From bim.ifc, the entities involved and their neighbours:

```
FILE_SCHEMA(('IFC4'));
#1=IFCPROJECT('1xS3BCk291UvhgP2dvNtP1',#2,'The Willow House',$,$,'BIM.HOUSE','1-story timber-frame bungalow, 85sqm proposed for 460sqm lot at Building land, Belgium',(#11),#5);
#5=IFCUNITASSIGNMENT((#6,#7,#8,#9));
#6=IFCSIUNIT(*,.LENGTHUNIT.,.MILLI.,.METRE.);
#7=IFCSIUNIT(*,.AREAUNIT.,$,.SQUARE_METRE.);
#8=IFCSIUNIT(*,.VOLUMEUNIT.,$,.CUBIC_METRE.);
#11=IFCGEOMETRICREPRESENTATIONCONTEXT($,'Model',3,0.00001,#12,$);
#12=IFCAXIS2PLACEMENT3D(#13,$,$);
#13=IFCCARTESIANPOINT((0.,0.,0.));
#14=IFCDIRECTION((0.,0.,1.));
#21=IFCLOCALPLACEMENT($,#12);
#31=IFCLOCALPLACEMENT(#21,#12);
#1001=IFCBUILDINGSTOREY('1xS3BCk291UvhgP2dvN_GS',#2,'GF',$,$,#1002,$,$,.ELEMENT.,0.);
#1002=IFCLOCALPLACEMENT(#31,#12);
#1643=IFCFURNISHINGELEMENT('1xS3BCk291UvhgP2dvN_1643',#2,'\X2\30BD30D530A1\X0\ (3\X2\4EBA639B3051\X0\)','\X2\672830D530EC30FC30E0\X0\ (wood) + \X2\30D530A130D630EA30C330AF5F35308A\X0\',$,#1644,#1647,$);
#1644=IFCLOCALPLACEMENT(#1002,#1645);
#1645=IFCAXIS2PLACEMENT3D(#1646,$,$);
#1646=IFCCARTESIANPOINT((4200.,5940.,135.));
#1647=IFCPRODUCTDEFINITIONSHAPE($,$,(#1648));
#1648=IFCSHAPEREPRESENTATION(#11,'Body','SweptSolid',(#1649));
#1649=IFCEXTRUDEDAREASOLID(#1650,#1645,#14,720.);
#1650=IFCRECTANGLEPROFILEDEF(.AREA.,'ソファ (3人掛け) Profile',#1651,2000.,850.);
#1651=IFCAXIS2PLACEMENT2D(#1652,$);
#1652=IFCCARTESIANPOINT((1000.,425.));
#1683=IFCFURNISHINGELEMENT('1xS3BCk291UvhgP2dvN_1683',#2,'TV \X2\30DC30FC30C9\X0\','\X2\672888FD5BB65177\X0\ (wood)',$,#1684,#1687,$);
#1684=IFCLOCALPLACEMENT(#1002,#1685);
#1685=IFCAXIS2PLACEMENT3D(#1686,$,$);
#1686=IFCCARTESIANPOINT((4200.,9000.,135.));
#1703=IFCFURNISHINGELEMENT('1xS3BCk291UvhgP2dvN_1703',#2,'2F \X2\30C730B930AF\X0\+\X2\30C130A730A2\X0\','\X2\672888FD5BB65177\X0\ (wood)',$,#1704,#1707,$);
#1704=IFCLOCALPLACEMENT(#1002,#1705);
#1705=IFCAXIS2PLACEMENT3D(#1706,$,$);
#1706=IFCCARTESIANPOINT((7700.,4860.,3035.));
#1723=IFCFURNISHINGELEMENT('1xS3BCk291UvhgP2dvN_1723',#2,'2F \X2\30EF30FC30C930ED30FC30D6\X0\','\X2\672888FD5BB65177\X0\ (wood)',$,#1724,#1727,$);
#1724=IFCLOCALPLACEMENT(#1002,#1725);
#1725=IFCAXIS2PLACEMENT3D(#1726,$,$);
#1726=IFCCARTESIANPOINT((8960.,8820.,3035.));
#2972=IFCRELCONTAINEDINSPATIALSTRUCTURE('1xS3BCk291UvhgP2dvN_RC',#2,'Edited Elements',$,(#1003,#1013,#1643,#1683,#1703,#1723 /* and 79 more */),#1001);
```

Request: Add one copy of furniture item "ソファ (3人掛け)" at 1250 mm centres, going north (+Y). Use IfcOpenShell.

```python
import numpy as np
import ifcopenshell
import ifcopenshell.api.geometry
import ifcopenshell.api.root
import ifcopenshell.util.element
import ifcopenshell.util.placement

model = ifcopenshell.open("bim.ifc")


def reuse_history(source, copy):
    """copy_class also copies each property set's owner history, people and application; keep the originals."""
    for rel in copy.IsDefinedBy:
        if rel.is_a("IfcRelDefinesByProperties") and (history := rel.RelatingPropertyDefinition.OwnerHistory):
            rel.RelatingPropertyDefinition.OwnerHistory = source.OwnerHistory
            ifcopenshell.util.element.remove_deep2(model, history)


source = model.by_id(1643)
base = ifcopenshell.util.placement.get_local_placement(source.ObjectPlacement)
step = np.array([0.0, 1.0, 0.0]) * 1250.0

for i in range(1, 2):
    copy = ifcopenshell.api.root.copy_class(model, product=source)
    copy.Representation = ifcopenshell.util.element.copy_deep(
        model, source.Representation, exclude=["IfcGeometricRepresentationContext", "IfcRepresentationMap"]
    )
    reuse_history(source, copy)
    matrix = base.copy()
    matrix[:3, 3] += i * step
    print("added at", matrix[:3, 3].round(3) + 0.0)
    ifcopenshell.api.geometry.edit_object_placement(model, product=copy, matrix=matrix, is_si=False)

model.write("bim_updated.ifc")
```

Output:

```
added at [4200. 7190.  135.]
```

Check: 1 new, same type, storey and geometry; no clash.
